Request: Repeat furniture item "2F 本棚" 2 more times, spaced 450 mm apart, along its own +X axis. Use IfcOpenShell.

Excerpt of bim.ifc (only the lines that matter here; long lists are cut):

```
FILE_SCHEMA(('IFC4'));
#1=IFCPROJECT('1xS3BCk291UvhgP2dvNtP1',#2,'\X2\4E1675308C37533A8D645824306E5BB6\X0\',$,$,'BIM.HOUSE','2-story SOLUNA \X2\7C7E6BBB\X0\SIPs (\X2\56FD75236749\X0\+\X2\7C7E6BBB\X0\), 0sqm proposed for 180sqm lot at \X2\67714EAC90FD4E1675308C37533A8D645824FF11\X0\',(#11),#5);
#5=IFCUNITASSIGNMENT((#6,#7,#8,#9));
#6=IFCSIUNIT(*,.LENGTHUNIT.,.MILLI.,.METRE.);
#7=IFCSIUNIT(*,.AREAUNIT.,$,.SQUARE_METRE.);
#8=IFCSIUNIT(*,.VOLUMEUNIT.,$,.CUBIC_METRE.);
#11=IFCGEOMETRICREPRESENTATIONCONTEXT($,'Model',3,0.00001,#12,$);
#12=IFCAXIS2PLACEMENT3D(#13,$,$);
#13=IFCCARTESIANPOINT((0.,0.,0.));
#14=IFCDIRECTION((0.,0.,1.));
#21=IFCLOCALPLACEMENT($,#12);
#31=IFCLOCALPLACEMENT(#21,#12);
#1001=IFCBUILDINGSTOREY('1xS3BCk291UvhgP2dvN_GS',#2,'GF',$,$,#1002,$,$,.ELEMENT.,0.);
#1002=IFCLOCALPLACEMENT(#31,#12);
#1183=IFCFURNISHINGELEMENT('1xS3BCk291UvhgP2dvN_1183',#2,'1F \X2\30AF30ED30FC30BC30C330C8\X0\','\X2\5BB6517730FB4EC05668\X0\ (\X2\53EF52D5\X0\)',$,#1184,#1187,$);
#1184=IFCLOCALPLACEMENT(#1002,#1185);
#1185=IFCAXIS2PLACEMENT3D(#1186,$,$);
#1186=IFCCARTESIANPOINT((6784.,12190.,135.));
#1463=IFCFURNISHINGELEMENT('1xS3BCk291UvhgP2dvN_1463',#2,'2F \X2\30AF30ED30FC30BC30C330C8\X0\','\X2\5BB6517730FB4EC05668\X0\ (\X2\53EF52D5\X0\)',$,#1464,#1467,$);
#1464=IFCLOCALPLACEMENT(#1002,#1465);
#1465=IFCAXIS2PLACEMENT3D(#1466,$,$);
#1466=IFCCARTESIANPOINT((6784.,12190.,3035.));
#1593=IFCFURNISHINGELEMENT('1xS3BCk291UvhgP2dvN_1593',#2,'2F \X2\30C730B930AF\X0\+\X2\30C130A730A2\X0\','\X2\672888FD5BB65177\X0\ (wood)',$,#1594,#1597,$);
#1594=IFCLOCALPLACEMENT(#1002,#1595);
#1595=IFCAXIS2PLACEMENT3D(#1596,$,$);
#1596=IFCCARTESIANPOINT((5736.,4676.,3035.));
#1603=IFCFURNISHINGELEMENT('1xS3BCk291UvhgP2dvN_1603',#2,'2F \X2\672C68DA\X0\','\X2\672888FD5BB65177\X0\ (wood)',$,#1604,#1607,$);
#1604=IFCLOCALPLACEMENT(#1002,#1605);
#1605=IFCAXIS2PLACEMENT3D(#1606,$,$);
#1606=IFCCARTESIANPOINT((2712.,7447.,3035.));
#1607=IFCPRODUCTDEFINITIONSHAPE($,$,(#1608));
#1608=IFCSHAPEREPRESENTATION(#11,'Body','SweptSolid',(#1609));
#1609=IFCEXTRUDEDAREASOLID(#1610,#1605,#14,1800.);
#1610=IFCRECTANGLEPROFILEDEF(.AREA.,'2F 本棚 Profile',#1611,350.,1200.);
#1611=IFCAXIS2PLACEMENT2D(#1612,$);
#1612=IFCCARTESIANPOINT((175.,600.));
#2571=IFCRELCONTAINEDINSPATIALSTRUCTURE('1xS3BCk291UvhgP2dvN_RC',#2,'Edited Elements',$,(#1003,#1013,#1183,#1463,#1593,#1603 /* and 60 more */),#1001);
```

```python
import ifcopenshell
import ifcopenshell.api.geometry
import ifcopenshell.api.root
import ifcopenshell.util.element
import ifcopenshell.util.placement
import ifcopenshell.util.unit

model = ifcopenshell.open("bim.ifc")
unit_scale = ifcopenshell.util.unit.calculate_unit_scale(model)


def reuse_history(source, copy):
    """copy_class also copies each property set's owner history, people and application; keep the originals."""
    for rel in copy.IsDefinedBy:
        if rel.is_a("IfcRelDefinesByProperties") and (history := rel.RelatingPropertyDefinition.OwnerHistory):
            rel.RelatingPropertyDefinition.OwnerHistory = source.OwnerHistory
            ifcopenshell.util.element.remove_deep2(model, history)


source = model.by_id(1603)
base = ifcopenshell.util.placement.get_local_placement(source.ObjectPlacement)
step = base[:3, 0] * 0.45 / unit_scale

for i in range(1, 3):
    copy = ifcopenshell.api.root.copy_class(model, product=source)
    copy.Representation = ifcopenshell.util.element.copy_deep(
        model, source.Representation, exclude=["IfcGeometricRepresentationContext", "IfcRepresentationMap"]
    )
    reuse_history(source, copy)
    matrix = base.copy()
    matrix[:3, 3] += i * step
    print("added at", matrix[:3, 3].round(3) + 0.0)
    ifcopenshell.api.geometry.edit_object_placement(model, product=copy, matrix=matrix, is_si=False)

model.write("bim_rev.ifc")
```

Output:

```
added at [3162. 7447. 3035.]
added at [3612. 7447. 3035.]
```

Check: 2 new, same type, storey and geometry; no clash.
